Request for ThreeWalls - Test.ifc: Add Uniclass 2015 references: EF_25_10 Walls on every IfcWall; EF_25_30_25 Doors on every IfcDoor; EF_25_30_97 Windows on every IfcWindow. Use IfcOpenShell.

First a look at what the model holds.

```python
import ifcopenshell

model = ifcopenshell.open("ThreeWalls - Test.ifc")
print(model.schema)
print("classifications:", [c.Name for c in model.by_type("IfcClassification")])
for ifc_class in ("IfcDoor", "IfcRoof", "IfcStair", "IfcWall", "IfcWindow"):
    print(ifc_class, len(model.by_type(ifc_class)))
```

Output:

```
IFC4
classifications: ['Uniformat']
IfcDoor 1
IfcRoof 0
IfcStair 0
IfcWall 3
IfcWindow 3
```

```python
import ifcopenshell
import ifcopenshell.api.classification

model = ifcopenshell.open("ThreeWalls - Test.ifc")

system = ifcopenshell.api.classification.add_classification(model, classification="Uniclass 2015")

codes = {
    "IfcWall": ("EF_25_10", "Walls"),
    "IfcDoor": ("EF_25_30_25", "Doors"),
    "IfcWindow": ("EF_25_30_97", "Windows"),
}
for ifc_class, (code, name) in codes.items():
    products = model.by_type(ifc_class)
    ifcopenshell.api.classification.add_reference(
        model, products=products, classification=system, identification=code, name=name
    )
    print(code, len(products))

model.write("ThreeWalls - Test-out.ifc")
```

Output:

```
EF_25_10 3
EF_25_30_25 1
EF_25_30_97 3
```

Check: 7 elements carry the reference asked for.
